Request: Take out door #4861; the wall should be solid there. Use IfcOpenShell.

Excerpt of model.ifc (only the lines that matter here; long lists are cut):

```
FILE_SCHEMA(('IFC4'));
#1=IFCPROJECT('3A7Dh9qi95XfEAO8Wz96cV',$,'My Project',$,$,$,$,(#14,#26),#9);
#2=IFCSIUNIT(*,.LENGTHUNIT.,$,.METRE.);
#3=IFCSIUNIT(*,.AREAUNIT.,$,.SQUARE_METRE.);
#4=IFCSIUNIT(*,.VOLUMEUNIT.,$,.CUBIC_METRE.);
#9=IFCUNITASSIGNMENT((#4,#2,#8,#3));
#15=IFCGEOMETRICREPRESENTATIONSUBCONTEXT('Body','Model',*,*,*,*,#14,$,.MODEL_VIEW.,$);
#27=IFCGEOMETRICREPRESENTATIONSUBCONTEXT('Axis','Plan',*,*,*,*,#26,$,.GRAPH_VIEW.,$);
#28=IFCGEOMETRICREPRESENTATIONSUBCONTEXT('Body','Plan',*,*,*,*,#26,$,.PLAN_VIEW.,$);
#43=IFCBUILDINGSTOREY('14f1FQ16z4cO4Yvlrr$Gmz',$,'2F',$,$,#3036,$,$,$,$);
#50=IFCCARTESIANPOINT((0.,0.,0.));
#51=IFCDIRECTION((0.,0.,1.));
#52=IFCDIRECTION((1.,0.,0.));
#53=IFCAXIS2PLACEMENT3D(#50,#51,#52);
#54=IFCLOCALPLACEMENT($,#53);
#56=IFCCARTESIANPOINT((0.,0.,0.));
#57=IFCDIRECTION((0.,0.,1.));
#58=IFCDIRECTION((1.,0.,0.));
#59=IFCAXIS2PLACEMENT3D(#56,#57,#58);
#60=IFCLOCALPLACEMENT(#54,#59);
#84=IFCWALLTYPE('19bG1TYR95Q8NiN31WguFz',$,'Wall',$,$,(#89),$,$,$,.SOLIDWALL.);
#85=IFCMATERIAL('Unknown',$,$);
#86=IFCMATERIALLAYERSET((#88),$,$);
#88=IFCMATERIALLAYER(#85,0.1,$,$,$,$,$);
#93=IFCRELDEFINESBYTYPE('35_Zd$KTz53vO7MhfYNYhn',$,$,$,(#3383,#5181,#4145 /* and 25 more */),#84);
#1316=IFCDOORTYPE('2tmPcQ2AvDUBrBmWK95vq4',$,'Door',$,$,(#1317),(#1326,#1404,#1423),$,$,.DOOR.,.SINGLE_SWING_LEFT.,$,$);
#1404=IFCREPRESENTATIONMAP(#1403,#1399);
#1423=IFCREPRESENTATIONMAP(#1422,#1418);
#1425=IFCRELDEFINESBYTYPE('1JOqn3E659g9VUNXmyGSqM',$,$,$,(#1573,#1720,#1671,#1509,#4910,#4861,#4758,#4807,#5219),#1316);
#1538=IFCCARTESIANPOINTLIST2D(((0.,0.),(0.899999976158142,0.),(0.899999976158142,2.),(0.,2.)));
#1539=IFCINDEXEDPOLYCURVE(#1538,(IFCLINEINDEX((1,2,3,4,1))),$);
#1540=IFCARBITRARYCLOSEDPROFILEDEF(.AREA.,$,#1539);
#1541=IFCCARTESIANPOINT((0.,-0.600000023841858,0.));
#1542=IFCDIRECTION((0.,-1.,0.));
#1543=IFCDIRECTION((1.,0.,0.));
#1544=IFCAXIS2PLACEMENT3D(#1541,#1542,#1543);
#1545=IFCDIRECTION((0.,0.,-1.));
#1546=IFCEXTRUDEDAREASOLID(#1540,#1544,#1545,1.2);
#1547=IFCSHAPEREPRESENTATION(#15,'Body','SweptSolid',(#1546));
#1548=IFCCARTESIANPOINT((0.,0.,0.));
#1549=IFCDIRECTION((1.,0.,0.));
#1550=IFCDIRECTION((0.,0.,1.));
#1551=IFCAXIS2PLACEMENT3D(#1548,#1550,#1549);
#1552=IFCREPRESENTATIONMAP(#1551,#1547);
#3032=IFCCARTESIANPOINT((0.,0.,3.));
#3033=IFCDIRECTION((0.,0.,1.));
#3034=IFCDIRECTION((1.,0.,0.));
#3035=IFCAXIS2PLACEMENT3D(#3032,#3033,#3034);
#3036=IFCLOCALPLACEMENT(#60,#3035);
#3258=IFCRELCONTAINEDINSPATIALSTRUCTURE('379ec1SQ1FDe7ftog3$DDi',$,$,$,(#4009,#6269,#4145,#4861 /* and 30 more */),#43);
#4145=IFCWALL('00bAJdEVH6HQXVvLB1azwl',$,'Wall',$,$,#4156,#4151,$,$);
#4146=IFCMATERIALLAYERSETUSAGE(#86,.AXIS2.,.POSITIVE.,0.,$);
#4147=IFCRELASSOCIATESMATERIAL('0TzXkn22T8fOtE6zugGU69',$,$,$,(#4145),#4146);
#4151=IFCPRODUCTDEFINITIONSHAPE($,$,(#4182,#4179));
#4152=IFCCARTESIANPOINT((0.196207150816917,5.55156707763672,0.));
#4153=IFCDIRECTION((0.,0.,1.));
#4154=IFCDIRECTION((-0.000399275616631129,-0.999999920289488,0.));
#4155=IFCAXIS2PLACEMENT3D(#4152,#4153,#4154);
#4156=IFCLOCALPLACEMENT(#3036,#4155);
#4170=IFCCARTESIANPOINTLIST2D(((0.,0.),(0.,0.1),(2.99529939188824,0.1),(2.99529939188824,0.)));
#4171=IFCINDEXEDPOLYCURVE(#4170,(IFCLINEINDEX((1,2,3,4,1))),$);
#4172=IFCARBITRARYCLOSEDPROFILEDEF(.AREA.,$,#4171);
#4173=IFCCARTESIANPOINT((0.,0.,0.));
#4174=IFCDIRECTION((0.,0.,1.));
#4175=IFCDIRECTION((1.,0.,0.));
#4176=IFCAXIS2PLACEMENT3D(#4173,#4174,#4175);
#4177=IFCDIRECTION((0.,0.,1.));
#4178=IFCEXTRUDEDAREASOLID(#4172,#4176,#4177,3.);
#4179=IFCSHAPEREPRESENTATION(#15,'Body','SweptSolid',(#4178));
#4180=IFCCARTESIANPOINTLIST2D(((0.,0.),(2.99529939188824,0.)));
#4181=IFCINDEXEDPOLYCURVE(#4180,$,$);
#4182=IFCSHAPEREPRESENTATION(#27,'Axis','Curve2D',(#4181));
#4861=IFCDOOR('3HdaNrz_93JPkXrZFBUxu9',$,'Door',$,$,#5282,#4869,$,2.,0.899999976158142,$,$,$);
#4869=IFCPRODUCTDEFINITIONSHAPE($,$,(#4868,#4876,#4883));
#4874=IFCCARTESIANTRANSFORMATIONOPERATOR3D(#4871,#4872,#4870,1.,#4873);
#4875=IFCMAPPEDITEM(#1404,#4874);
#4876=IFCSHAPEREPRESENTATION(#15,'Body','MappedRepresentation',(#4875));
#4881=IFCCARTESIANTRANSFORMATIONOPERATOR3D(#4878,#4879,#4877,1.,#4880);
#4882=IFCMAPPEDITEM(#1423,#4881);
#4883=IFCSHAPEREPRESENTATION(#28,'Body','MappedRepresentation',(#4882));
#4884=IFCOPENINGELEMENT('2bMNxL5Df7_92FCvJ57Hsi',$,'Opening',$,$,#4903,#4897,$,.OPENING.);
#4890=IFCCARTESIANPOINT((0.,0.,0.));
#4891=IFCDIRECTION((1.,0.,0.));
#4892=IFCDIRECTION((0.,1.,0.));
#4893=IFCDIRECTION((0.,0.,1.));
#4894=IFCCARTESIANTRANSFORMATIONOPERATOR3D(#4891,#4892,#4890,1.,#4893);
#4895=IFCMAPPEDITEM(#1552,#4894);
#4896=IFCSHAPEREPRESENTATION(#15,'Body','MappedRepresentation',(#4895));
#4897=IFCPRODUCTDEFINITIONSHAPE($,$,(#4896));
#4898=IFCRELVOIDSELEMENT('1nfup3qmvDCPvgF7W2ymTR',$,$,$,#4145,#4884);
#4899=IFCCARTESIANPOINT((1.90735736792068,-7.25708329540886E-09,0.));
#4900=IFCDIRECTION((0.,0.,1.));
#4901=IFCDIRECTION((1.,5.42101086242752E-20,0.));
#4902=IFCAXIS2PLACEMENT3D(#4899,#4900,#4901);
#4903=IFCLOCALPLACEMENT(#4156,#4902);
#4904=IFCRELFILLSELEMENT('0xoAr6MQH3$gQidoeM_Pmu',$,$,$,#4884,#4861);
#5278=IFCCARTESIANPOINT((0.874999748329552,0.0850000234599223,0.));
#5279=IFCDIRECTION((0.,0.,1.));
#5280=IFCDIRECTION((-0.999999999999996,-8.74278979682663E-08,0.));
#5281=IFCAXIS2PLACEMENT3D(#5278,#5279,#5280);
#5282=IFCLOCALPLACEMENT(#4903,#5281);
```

```python
import ifcopenshell
import ifcopenshell.api.feature
import ifcopenshell.api.root
import ifcopenshell.geom
import ifcopenshell.util.shape

model = ifcopenshell.open("model.ifc")
settings = ifcopenshell.geom.settings()


def volume(element):
    """Net volume in cubic metres, openings subtracted."""
    shape = ifcopenshell.geom.create_shape(settings, element)
    return ifcopenshell.util.shape.get_volume(shape.geometry)


door = model.by_guid("3HdaNrz_93JPkXrZFBUxu9")
opening = door.FillsVoids[0].RelatingOpeningElement
wall = opening.VoidsElements[0].RelatingBuildingElement
before = volume(wall)

ifcopenshell.api.root.remove_product(model, product=door)
ifcopenshell.api.feature.remove_feature(model, feature=opening)

after = volume(wall)

print(f"wall volume {before:.3f} -> {after:.3f} m3")

model.write("model_v2.ifc")
```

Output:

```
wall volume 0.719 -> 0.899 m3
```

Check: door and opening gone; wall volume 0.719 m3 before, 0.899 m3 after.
